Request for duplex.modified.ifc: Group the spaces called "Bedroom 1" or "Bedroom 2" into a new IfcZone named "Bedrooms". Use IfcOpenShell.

First a look at what the model holds.

```python
import ifcopenshell

model = ifcopenshell.open("duplex.modified.ifc")
print(model.schema)
seen = {}
for space in model.by_type("IfcSpace"):
    seen[space.LongName] = seen.get(space.LongName, 0) + 1
for name, count in sorted(seen.items(), key=str):
    print(count, "x", name)
print("zones:", [z.Name for z in model.by_type("IfcZone")][:20])
```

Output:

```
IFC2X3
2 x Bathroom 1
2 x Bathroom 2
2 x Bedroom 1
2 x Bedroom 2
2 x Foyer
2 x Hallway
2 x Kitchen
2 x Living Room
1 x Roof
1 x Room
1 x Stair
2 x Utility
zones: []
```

```python
import ifcopenshell
import ifcopenshell.api.group
import ifcopenshell.api.root

model = ifcopenshell.open("duplex.modified.ifc")

names = {"Bedroom 1", "Bedroom 2"}
spaces = [s for s in model.by_type("IfcSpace") if s.LongName in names]

zone = ifcopenshell.api.root.create_entity(model, ifc_class="IfcZone", name="Bedrooms")
ifcopenshell.api.group.assign_group(model, products=spaces, group=zone)
print(len(spaces), "spaces in", zone.Name)

model.write("duplex.modified_updated.ifc")
```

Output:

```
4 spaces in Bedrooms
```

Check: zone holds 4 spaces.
